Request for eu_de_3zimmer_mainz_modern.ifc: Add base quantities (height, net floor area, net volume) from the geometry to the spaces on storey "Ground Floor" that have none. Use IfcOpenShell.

First a look at what the model holds.

```python
import ifcopenshell
import ifcopenshell.util.element
import ifcopenshell.util.unit

model = ifcopenshell.open("eu_de_3zimmer_mainz_modern.ifc")
print(model.schema)
for unit_type in ("LENGTHUNIT", "AREAUNIT", "VOLUMEUNIT"):
    print(unit_type, ifcopenshell.util.unit.calculate_unit_scale(model, unit_type))
storey = next(s for s in model.by_type("IfcBuildingStorey") if s.Name == "Ground Floor")
spaces = [e for e in ifcopenshell.util.element.get_decomposition(storey) if e.is_a("IfcSpace")]
for e in sorted(spaces, key=lambda e: e.id()):
    print(e.id(), e.is_a(), e.Name, list(ifcopenshell.util.element.get_psets(e, qtos_only=True)), sep=" | ")
```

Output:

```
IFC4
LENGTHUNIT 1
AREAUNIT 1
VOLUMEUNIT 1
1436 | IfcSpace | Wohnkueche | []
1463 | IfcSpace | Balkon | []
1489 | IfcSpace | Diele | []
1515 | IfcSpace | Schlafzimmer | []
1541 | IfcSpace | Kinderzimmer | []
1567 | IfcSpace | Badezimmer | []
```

```python
import ifcopenshell
import ifcopenshell.api.pset
import ifcopenshell.geom
import ifcopenshell.util.element
import ifcopenshell.util.shape
import ifcopenshell.util.unit

model = ifcopenshell.open("eu_de_3zimmer_mainz_modern.ifc")
unit_scale = ifcopenshell.util.unit.calculate_unit_scale(model)
area_scale = ifcopenshell.util.unit.calculate_unit_scale(model, "AREAUNIT")
volume_scale = ifcopenshell.util.unit.calculate_unit_scale(model, "VOLUMEUNIT")
settings = ifcopenshell.geom.settings()

storey = next(s for s in model.by_type("IfcBuildingStorey") if s.Name == "Ground Floor")
spaces = [e for e in ifcopenshell.util.element.get_decomposition(storey) if e.is_a("IfcSpace")]

for e in sorted(spaces, key=lambda e: e.id()):
    if ifcopenshell.util.element.get_psets(e, qtos_only=True, should_inherit=False):
        continue
    # Geometry comes back in metres, in the element's own axes.
    shape = ifcopenshell.geom.create_shape(settings, e)
    values = {
        "Height": ifcopenshell.util.shape.get_z(shape.geometry) / unit_scale,
        "NetFloorArea": ifcopenshell.util.shape.get_footprint_area(shape.geometry) / area_scale,
        "NetVolume": ifcopenshell.util.shape.get_volume(shape.geometry) / volume_scale,
    }
    qto = ifcopenshell.api.pset.add_qto(model, product=e, name="Qto_SpaceBaseQuantities")
    ifcopenshell.api.pset.edit_qto(model, qto=qto, properties=values)
    print(e.id(), {k: round(v, 3) for k, v in values.items()})

model.write("eu_de_3zimmer_mainz_modern_edited.ifc")
```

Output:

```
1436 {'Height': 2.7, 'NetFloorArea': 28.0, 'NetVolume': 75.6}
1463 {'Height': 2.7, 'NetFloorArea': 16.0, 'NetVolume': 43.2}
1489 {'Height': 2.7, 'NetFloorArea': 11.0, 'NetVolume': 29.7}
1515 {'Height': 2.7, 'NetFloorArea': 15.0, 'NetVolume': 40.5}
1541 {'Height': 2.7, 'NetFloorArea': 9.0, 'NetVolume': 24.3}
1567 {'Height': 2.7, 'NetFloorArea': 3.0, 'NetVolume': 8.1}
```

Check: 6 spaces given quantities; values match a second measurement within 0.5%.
